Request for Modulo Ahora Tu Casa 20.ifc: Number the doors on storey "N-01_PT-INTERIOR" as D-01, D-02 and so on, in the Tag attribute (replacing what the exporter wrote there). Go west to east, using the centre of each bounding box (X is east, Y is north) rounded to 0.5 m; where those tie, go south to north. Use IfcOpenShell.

First a look at what the model holds.

```python
import ifcopenshell
import ifcopenshell.util.element
import ifcopenshell.util.placement

model = ifcopenshell.open("Modulo Ahora Tu Casa 20.ifc")
print(model.schema)
storey = next(s for s in model.by_type("IfcBuildingStorey") if s.Name == "N-01_PT-INTERIOR")
doors = [e for e in ifcopenshell.util.element.get_decomposition(storey) if e.is_a("IfcDoor")]
for e in sorted(doors, key=lambda e: e.id()):
    origin = ifcopenshell.util.placement.get_local_placement(e.ObjectPlacement)[:3, 3]
    print(e.id(), e.Tag, e.Name, origin.round(2) + 0.0, sep=" | ")
```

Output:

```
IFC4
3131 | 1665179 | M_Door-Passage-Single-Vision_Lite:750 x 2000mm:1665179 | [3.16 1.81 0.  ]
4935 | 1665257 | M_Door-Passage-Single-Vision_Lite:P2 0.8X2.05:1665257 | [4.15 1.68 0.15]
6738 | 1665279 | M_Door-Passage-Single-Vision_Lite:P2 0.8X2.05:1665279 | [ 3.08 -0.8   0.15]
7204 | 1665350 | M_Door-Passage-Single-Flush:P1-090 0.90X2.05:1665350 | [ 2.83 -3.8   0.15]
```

```python
import ifcopenshell
import ifcopenshell.geom
import ifcopenshell.util.element
import ifcopenshell.util.shape

model = ifcopenshell.open("Modulo Ahora Tu Casa 20.ifc")
settings = ifcopenshell.geom.settings()
settings.set("use-world-coords", True)


def centre(element):
    shape = ifcopenshell.geom.create_shape(settings, element)
    return ifcopenshell.util.shape.get_bbox_centroid(shape.geometry)


storey = next(s for s in model.by_type("IfcBuildingStorey") if s.Name == "N-01_PT-INTERIOR")
doors = [e for e in ifcopenshell.util.element.get_decomposition(storey) if e.is_a("IfcDoor")]

# Insertion points can sit at a corner or the storey origin, so sort by the geometry (in metres).
centres = {e: centre(e) for e in doors}
doors.sort(key=lambda e: (round(centres[e][0] / 0.5), centres[e][1]))

for i, e in enumerate(doors, start=1):
    number = f"D-{i:02d}"
    e.Tag = number
    print(e.id(), number)

model.write("Modulo Ahora Tu Casa 20_rev.ifc")
```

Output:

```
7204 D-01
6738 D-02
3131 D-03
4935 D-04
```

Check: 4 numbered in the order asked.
